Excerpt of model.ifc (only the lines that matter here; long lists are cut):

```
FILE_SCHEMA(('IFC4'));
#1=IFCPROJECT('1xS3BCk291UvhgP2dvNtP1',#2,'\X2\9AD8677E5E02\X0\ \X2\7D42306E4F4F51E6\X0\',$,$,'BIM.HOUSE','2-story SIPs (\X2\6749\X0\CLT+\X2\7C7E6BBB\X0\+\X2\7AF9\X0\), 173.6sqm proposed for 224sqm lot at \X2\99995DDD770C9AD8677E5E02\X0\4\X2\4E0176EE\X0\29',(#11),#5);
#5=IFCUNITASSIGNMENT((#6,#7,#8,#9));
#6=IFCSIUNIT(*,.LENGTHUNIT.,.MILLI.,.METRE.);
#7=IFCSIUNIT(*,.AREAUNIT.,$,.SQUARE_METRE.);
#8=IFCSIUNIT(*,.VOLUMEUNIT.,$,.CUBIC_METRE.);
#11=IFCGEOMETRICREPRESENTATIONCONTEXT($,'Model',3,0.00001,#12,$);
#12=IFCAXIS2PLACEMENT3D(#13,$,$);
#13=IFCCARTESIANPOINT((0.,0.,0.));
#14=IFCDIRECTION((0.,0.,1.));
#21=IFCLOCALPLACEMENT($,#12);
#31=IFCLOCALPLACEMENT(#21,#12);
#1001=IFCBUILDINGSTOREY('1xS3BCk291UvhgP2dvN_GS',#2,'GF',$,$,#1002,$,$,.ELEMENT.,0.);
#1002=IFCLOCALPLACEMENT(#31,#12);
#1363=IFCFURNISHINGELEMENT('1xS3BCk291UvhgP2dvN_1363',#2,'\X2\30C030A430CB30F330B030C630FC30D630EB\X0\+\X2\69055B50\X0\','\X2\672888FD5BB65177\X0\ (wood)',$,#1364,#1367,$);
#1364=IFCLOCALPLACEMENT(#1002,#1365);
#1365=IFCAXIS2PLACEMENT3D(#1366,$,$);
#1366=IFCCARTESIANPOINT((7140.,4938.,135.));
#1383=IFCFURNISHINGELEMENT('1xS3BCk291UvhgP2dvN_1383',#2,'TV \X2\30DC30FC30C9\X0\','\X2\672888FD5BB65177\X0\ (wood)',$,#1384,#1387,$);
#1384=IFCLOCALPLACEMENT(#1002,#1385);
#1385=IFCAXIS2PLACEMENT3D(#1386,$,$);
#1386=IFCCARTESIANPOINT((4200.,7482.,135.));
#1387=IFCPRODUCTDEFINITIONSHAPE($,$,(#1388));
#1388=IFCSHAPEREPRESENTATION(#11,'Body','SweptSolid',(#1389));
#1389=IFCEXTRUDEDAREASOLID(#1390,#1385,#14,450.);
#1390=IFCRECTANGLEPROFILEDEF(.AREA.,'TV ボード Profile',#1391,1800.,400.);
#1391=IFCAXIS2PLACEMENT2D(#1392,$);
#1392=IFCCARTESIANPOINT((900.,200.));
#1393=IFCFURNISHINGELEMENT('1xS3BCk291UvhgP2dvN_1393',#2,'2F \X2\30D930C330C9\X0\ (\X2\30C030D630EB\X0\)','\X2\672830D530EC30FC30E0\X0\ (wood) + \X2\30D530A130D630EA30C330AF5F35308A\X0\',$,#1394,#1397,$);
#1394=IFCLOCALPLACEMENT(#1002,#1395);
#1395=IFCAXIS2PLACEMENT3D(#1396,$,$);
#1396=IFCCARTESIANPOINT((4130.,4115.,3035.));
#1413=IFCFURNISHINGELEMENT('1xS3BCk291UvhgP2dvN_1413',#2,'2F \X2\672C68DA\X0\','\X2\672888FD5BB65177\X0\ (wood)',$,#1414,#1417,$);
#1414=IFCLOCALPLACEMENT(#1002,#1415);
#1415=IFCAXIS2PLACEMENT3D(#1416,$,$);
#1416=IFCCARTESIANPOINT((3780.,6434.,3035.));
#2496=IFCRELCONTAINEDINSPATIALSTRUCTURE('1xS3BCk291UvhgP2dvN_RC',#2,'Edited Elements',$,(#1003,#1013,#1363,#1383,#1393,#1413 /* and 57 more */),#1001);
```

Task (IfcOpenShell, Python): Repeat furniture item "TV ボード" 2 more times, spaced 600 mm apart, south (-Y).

```python
import numpy as np
import ifcopenshell
import ifcopenshell.api.geometry
import ifcopenshell.api.root
import ifcopenshell.util.element
import ifcopenshell.util.placement
import ifcopenshell.util.unit

model = ifcopenshell.open("model.ifc")
unit_scale = ifcopenshell.util.unit.calculate_unit_scale(model)


def reuse_history(source, copy):
    """copy_class also copies each property set's owner history, people and application; keep the originals."""
    for rel in copy.IsDefinedBy:
        if rel.is_a("IfcRelDefinesByProperties") and (history := rel.RelatingPropertyDefinition.OwnerHistory):
            rel.RelatingPropertyDefinition.OwnerHistory = source.OwnerHistory
            ifcopenshell.util.element.remove_deep2(model, history)


source = model.by_guid("1xS3BCk291UvhgP2dvN_1383")
base = ifcopenshell.util.placement.get_local_placement(source.ObjectPlacement)
step = np.array([0.0, -1.0, 0.0]) * 0.6 / unit_scale

for i in range(1, 3):
    copy = ifcopenshell.api.root.copy_class(model, product=source)
    copy.Representation = ifcopenshell.util.element.copy_deep(
        model, source.Representation, exclude=["IfcGeometricRepresentationContext", "IfcRepresentationMap"]
    )
    reuse_history(source, copy)
    matrix = base.copy()
    matrix[:3, 3] += i * step
    print("added at", matrix[:3, 3].round(3) + 0.0)
    ifcopenshell.api.geometry.edit_object_placement(model, product=copy, matrix=matrix, is_si=False)

model.write("model_edited.ifc")
```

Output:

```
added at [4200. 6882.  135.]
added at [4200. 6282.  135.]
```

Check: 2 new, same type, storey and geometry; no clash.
